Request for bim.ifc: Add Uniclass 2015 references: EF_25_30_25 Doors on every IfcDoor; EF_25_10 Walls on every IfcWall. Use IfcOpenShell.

First a look at what the model holds.

```python
import ifcopenshell

model = ifcopenshell.open("bim.ifc")
print(model.schema)
print("classifications:", [c.Name for c in model.by_type("IfcClassification")])
for ifc_class in ("IfcDoor", "IfcRoof", "IfcStair", "IfcWall", "IfcWindow"):
    print(ifc_class, len(model.by_type(ifc_class)))
```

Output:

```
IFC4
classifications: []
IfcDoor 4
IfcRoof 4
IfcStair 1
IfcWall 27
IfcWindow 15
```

```python
import ifcopenshell
import ifcopenshell.api.classification

model = ifcopenshell.open("bim.ifc")

system = ifcopenshell.api.classification.add_classification(model, classification="Uniclass 2015")

codes = {
    "IfcDoor": ("EF_25_30_25", "Doors"),
    "IfcWall": ("EF_25_10", "Walls"),
}
for ifc_class, (code, name) in codes.items():
    products = model.by_type(ifc_class)
    ifcopenshell.api.classification.add_reference(
        model, products=products, classification=system, identification=code, name=name
    )
    print(code, len(products))

model.write("bim_v2.ifc")
```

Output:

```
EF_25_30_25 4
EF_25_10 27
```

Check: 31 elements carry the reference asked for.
